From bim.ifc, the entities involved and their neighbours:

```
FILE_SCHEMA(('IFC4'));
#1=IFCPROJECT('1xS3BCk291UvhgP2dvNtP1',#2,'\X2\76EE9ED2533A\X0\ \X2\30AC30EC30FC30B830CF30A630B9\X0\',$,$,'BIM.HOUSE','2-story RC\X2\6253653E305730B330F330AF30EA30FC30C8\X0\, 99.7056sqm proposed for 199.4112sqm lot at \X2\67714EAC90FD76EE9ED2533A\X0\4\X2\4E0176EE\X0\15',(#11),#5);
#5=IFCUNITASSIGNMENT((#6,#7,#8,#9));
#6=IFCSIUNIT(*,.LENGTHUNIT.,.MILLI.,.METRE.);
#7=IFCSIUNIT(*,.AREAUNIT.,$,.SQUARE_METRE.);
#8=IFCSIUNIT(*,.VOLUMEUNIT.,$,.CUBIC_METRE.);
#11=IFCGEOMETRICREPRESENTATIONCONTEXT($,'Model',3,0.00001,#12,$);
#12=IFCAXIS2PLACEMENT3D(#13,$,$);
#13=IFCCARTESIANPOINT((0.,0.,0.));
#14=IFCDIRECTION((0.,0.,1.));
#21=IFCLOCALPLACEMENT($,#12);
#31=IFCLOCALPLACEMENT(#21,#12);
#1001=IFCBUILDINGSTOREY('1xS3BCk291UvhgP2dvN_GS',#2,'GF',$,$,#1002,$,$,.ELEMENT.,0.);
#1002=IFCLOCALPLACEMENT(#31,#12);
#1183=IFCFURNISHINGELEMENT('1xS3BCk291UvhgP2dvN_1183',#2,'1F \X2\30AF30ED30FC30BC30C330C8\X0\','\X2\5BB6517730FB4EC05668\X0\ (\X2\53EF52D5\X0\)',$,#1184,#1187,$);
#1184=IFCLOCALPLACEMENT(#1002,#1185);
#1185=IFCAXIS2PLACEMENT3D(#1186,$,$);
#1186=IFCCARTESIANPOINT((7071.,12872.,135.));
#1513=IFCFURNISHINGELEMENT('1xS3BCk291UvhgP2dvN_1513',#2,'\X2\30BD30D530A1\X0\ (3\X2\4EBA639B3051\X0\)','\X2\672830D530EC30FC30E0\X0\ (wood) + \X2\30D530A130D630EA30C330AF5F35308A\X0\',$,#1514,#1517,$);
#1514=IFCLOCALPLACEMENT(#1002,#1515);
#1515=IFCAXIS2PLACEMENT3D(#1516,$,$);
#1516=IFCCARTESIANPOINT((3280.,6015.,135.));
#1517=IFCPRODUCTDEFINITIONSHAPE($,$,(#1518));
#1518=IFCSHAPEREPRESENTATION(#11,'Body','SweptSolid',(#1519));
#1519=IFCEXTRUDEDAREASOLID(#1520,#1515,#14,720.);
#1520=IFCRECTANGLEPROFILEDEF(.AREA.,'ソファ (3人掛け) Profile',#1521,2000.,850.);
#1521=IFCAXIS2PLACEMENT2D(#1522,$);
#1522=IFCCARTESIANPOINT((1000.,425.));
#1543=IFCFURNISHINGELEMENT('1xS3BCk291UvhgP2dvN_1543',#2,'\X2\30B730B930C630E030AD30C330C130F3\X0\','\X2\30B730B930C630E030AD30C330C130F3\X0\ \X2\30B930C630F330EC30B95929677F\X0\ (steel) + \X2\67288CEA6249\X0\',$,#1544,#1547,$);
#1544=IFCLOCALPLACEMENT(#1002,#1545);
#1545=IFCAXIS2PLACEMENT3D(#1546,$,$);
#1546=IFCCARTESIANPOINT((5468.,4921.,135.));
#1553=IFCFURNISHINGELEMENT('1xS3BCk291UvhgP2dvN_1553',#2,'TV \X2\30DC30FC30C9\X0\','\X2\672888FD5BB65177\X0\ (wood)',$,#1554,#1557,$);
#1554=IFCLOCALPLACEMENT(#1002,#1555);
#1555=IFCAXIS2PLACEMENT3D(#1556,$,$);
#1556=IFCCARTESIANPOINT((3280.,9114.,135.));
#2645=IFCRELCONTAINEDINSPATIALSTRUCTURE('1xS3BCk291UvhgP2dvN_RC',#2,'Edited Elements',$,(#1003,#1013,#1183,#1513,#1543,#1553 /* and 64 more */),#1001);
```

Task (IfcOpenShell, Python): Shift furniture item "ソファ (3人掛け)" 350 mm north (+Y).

```python
import ifcopenshell
import ifcopenshell.api.geometry
import ifcopenshell.util.placement
import ifcopenshell.util.unit

model = ifcopenshell.open("bim.ifc")
unit_scale = ifcopenshell.util.unit.calculate_unit_scale(model)

item = model.by_guid("1xS3BCk291UvhgP2dvN_1513")
matrix = ifcopenshell.util.placement.get_local_placement(item.ObjectPlacement)
matrix[1, 3] += 0.35 / unit_scale
ifcopenshell.api.geometry.edit_object_placement(model, product=item, matrix=matrix, is_si=False)

print(ifcopenshell.util.placement.get_local_placement(item.ObjectPlacement).round(3) + 0.0)

model.write("bim_rev.ifc")
```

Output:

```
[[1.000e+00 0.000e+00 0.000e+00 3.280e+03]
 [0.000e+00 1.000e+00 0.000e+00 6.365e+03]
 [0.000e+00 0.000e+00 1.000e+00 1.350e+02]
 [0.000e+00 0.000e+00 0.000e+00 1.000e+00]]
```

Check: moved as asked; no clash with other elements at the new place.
